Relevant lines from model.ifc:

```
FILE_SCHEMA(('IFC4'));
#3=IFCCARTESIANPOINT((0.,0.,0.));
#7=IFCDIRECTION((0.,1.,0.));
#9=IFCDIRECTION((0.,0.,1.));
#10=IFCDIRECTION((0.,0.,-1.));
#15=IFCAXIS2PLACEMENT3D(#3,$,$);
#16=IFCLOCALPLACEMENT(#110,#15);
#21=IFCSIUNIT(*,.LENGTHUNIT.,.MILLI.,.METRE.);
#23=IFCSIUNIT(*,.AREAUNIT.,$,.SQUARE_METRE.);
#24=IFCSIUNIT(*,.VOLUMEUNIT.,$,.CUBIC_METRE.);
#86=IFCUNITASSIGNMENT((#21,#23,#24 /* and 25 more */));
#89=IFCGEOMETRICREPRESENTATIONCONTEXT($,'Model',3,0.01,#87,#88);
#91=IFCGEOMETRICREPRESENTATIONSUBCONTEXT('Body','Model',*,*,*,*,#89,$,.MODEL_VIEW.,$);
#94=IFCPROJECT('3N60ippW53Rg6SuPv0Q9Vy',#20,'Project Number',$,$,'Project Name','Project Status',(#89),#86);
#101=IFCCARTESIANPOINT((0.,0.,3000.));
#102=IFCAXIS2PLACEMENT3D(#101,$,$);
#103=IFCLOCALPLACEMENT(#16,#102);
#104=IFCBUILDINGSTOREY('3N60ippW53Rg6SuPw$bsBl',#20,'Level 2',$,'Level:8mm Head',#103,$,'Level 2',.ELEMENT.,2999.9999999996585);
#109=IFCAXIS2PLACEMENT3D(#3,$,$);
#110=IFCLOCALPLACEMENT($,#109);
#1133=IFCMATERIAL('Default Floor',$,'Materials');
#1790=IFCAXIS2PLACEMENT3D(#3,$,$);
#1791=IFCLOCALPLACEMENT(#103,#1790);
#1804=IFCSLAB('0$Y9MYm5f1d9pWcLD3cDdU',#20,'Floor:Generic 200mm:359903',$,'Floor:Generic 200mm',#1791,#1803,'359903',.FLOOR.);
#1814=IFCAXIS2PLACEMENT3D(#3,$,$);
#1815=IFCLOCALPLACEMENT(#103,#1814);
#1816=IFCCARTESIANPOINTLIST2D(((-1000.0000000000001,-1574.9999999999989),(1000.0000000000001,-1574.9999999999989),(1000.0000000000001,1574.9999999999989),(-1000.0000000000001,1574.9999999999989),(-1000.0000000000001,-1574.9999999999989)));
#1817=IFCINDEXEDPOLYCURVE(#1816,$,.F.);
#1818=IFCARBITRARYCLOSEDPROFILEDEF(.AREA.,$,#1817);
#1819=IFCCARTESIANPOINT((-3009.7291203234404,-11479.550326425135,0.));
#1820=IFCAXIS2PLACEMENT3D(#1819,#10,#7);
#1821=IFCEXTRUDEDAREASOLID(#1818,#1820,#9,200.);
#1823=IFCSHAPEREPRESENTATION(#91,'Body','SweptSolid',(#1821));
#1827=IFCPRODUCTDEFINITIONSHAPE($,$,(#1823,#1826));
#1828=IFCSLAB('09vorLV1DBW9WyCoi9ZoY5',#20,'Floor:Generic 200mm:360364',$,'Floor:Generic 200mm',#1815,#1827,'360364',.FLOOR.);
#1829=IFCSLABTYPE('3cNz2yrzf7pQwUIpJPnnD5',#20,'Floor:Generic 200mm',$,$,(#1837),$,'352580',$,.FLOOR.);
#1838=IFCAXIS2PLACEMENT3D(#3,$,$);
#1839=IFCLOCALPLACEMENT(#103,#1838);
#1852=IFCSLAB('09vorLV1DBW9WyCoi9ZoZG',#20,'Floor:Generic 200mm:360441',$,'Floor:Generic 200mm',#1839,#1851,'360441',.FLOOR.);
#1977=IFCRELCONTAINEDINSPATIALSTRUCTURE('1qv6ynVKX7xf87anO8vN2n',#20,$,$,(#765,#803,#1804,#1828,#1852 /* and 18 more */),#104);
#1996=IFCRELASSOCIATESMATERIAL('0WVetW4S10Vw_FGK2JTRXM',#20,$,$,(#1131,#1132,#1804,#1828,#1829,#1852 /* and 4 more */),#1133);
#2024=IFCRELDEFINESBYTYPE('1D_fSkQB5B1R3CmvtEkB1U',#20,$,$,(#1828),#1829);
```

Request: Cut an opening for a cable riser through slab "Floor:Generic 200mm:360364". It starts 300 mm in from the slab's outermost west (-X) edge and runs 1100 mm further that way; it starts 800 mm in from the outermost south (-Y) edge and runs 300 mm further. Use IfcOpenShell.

```python
import numpy as np
import ifcopenshell
import ifcopenshell.api.feature
import ifcopenshell.api.geometry
import ifcopenshell.api.root
import ifcopenshell.geom
import ifcopenshell.util.placement
import ifcopenshell.util.representation
import ifcopenshell.util.shape
import ifcopenshell.util.unit

model = ifcopenshell.open("model.ifc")
unit_scale = ifcopenshell.util.unit.calculate_unit_scale(model)
settings = ifcopenshell.geom.settings()


def volume(element):
    """Net volume in cubic metres, openings subtracted."""
    shape = ifcopenshell.geom.create_shape(settings, element)
    return ifcopenshell.util.shape.get_volume(shape.geometry)


slab = model.by_guid("09vorLV1DBW9WyCoi9ZoY5")
before = volume(slab)

# Extent in the slab's own axes, in metres. The edges named are its -X and -Y sides.
slab_shape = ifcopenshell.geom.create_shape(settings, slab)
vertices = ifcopenshell.util.shape.get_vertices(slab_shape.geometry)
x_min, y_min, bottom = vertices.min(axis=0)
top = vertices[:, 2].max()

opening = ifcopenshell.api.root.create_entity(model, ifc_class="IfcOpeningElement", name="Cable riser opening", predefined_type="OPENING")
context = ifcopenshell.util.representation.get_context(model, "Model", "Body", "MODEL_VIEW")
width, depth = 1.1, 0.3
outline = [(0.0, 0.0), (width, 0.0), (width, depth), (0.0, depth), (0.0, 0.0)]
# Overshoot both faces by 50 mm so the cut is clean.
shape = ifcopenshell.api.geometry.add_slab_representation(
    model, context=context, depth=top - bottom + 0.1, polyline=outline
)
ifcopenshell.api.geometry.assign_representation(model, product=opening, representation=shape)

matrix = ifcopenshell.util.placement.get_local_placement(slab.ObjectPlacement)
matrix[:, 3] = matrix @ np.append(np.array([x_min + 0.3, y_min + 0.8, bottom - 0.05]) / unit_scale, 1.0)
ifcopenshell.api.geometry.edit_object_placement(model, product=opening, matrix=matrix, is_si=False)
ifcopenshell.api.feature.add_feature(model, feature=opening, element=slab)

after = volume(slab)

print(f"slab volume {before:.3f} -> {after:.3f} m3")

model.write("model_rev.ifc")
```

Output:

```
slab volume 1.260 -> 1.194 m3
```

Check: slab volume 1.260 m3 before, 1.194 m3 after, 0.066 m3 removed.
